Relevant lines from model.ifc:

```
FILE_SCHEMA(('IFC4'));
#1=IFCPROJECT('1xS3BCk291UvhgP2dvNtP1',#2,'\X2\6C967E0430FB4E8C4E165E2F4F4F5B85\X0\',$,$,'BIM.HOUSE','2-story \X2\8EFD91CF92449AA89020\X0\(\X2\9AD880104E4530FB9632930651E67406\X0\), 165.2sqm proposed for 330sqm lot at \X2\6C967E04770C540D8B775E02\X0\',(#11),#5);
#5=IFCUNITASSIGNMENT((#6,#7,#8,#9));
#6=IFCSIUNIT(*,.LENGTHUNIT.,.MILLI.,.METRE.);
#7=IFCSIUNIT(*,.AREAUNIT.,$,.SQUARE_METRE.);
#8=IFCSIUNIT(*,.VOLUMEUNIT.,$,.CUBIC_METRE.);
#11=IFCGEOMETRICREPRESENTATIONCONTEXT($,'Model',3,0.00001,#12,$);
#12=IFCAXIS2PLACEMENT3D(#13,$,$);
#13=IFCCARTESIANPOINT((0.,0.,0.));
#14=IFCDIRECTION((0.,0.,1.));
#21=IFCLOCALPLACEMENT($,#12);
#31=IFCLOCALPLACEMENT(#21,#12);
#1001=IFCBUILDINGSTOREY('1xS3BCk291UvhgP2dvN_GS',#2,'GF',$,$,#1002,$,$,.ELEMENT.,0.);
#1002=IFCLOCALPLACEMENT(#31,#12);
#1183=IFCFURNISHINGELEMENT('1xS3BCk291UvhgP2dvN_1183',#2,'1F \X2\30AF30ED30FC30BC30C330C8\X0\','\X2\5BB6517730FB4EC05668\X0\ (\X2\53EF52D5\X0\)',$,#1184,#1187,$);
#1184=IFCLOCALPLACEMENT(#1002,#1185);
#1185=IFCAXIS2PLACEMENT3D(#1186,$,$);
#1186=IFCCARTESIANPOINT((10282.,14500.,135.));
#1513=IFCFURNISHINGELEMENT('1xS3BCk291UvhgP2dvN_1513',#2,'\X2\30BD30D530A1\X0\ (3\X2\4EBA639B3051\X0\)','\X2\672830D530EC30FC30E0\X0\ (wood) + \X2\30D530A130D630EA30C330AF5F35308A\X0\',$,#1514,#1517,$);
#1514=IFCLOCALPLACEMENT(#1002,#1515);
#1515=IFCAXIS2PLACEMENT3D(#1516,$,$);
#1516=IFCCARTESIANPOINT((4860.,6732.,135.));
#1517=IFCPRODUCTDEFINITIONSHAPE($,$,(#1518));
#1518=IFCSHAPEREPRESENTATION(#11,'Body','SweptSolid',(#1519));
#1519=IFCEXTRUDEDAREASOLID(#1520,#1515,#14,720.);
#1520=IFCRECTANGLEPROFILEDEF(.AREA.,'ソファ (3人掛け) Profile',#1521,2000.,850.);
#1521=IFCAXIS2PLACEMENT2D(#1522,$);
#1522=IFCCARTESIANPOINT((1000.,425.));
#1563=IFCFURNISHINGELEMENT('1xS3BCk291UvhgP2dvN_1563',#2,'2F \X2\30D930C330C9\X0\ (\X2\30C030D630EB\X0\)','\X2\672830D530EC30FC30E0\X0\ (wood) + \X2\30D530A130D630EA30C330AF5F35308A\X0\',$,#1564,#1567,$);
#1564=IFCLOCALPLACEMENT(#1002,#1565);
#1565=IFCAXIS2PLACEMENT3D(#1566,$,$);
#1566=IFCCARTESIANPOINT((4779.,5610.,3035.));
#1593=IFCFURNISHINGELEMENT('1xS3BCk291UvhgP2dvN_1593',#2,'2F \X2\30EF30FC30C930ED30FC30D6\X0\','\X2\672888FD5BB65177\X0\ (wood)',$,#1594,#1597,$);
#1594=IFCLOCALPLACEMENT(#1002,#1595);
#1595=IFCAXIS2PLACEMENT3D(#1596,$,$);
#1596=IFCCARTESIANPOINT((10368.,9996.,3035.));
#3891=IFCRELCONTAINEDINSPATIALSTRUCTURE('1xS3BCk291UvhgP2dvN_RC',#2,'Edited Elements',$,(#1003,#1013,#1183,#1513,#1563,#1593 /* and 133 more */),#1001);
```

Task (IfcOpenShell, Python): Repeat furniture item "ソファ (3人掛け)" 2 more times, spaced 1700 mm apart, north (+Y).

```python
import numpy as np
import ifcopenshell
import ifcopenshell.api.geometry
import ifcopenshell.api.root
import ifcopenshell.util.element
import ifcopenshell.util.placement

model = ifcopenshell.open("model.ifc")


def reuse_history(source, copy):
    """copy_class also copies each property set's owner history, people and application; keep the originals."""
    for rel in copy.IsDefinedBy:
        if rel.is_a("IfcRelDefinesByProperties") and (history := rel.RelatingPropertyDefinition.OwnerHistory):
            rel.RelatingPropertyDefinition.OwnerHistory = source.OwnerHistory
            ifcopenshell.util.element.remove_deep2(model, history)


source = model.by_guid("1xS3BCk291UvhgP2dvN_1513")
base = ifcopenshell.util.placement.get_local_placement(source.ObjectPlacement)
step = np.array([0.0, 1.0, 0.0]) * 1700.0

for i in range(1, 3):
    copy = ifcopenshell.api.root.copy_class(model, product=source)
    copy.Representation = ifcopenshell.util.element.copy_deep(
        model, source.Representation, exclude=["IfcGeometricRepresentationContext", "IfcRepresentationMap"]
    )
    reuse_history(source, copy)
    matrix = base.copy()
    matrix[:3, 3] += i * step
    print("added at", matrix[:3, 3].round(3) + 0.0)
    ifcopenshell.api.geometry.edit_object_placement(model, product=copy, matrix=matrix, is_si=False)

model.write("model_rev.ifc")
```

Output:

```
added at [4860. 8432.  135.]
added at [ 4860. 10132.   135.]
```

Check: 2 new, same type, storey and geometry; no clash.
